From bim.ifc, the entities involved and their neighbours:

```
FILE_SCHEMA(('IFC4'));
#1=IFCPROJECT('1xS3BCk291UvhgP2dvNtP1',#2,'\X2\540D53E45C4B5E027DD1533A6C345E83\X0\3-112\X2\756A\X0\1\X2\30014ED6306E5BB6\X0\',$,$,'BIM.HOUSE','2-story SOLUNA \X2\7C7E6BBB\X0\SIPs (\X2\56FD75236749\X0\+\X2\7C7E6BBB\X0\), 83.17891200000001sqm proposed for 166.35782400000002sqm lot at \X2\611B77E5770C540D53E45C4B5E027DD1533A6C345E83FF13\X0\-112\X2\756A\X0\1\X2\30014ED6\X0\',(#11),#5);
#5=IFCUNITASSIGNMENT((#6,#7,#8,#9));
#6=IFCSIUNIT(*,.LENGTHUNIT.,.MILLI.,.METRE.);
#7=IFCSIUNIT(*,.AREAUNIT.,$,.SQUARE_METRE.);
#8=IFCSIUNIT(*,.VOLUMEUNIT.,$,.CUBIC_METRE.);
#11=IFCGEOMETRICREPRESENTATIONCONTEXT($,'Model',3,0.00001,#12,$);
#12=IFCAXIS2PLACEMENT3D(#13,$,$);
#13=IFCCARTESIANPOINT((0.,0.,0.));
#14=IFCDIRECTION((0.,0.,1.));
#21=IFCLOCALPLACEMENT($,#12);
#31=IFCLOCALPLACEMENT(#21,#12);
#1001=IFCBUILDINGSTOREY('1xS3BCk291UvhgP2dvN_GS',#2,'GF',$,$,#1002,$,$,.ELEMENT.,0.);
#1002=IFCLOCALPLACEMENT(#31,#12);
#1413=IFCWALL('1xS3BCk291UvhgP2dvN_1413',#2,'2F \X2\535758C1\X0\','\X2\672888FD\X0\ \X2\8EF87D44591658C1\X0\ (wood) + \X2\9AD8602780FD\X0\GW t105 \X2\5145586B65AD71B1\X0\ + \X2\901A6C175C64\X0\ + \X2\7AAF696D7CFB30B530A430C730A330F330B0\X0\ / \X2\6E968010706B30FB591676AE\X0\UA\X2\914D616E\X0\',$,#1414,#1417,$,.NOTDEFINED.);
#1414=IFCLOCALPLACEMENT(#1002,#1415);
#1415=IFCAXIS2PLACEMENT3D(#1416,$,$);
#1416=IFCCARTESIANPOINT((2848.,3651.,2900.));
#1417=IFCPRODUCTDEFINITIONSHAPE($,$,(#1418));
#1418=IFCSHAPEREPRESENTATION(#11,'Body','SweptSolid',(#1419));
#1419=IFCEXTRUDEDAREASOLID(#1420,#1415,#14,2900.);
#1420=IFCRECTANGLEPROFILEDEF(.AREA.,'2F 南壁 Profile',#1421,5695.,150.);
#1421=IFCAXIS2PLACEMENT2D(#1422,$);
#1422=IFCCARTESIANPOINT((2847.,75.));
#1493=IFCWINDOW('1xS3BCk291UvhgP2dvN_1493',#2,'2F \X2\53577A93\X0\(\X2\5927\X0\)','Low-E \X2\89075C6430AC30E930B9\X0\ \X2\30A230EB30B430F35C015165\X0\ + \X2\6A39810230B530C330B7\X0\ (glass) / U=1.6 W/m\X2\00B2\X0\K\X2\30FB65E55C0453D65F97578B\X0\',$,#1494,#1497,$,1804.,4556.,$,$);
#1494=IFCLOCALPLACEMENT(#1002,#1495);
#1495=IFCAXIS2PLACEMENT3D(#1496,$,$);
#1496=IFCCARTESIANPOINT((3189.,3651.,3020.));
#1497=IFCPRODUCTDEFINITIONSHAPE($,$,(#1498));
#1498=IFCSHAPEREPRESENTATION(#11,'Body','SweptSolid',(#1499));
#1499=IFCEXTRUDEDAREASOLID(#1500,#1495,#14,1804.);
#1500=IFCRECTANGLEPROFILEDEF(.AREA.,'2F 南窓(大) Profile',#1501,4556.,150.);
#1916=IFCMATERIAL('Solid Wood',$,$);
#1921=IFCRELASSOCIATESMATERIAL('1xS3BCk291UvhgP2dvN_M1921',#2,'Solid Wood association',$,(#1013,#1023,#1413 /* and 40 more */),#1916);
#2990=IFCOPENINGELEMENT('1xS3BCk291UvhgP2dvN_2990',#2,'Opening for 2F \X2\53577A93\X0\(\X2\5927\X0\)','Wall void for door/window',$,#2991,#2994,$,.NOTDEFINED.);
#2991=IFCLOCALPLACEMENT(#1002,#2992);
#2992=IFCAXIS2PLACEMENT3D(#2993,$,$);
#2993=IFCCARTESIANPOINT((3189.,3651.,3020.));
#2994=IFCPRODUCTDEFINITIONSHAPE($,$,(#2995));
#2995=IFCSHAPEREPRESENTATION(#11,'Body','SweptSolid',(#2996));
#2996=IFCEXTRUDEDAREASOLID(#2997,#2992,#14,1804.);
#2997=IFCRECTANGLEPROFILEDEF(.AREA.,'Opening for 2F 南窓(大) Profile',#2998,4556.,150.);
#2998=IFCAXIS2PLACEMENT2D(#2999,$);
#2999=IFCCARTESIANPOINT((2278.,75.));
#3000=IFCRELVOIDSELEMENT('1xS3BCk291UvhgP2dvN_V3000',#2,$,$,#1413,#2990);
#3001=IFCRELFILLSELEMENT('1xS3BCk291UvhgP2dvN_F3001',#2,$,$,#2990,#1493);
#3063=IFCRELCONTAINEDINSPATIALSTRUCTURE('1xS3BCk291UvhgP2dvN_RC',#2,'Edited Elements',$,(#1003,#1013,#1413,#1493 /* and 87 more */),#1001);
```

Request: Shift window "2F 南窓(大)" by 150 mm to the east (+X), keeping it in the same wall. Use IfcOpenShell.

```python
import ifcopenshell
import ifcopenshell.api.geometry
import ifcopenshell.util.placement
import ifcopenshell.util.unit

model = ifcopenshell.open("bim.ifc")
unit_scale = ifcopenshell.util.unit.calculate_unit_scale(model)

window = model.by_guid("1xS3BCk291UvhgP2dvN_1493")
opening = window.FillsVoids[0].RelatingOpeningElement
wall = opening.VoidsElements[0].RelatingBuildingElement

wall_matrix = ifcopenshell.util.placement.get_local_placement(wall.ObjectPlacement)
shift = wall_matrix[:3, 0] * 0.15 / unit_scale
before = ifcopenshell.util.placement.get_local_placement(window.ObjectPlacement)[:3, 3].copy()

# The window is not placed relative to its opening, so move both.
for product in (opening, window):
    matrix = ifcopenshell.util.placement.get_local_placement(product.ObjectPlacement)
    matrix[:3, 3] += shift
    ifcopenshell.api.geometry.edit_object_placement(model, product=product, matrix=matrix, is_si=False)

after = ifcopenshell.util.placement.get_local_placement(window.ObjectPlacement)[:3, 3]
print("window moved by", (after - before).round(3) + 0.0)

model.write("bim_updated.ifc")
```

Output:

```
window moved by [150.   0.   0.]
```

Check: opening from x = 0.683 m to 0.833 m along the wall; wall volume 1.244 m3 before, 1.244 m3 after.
